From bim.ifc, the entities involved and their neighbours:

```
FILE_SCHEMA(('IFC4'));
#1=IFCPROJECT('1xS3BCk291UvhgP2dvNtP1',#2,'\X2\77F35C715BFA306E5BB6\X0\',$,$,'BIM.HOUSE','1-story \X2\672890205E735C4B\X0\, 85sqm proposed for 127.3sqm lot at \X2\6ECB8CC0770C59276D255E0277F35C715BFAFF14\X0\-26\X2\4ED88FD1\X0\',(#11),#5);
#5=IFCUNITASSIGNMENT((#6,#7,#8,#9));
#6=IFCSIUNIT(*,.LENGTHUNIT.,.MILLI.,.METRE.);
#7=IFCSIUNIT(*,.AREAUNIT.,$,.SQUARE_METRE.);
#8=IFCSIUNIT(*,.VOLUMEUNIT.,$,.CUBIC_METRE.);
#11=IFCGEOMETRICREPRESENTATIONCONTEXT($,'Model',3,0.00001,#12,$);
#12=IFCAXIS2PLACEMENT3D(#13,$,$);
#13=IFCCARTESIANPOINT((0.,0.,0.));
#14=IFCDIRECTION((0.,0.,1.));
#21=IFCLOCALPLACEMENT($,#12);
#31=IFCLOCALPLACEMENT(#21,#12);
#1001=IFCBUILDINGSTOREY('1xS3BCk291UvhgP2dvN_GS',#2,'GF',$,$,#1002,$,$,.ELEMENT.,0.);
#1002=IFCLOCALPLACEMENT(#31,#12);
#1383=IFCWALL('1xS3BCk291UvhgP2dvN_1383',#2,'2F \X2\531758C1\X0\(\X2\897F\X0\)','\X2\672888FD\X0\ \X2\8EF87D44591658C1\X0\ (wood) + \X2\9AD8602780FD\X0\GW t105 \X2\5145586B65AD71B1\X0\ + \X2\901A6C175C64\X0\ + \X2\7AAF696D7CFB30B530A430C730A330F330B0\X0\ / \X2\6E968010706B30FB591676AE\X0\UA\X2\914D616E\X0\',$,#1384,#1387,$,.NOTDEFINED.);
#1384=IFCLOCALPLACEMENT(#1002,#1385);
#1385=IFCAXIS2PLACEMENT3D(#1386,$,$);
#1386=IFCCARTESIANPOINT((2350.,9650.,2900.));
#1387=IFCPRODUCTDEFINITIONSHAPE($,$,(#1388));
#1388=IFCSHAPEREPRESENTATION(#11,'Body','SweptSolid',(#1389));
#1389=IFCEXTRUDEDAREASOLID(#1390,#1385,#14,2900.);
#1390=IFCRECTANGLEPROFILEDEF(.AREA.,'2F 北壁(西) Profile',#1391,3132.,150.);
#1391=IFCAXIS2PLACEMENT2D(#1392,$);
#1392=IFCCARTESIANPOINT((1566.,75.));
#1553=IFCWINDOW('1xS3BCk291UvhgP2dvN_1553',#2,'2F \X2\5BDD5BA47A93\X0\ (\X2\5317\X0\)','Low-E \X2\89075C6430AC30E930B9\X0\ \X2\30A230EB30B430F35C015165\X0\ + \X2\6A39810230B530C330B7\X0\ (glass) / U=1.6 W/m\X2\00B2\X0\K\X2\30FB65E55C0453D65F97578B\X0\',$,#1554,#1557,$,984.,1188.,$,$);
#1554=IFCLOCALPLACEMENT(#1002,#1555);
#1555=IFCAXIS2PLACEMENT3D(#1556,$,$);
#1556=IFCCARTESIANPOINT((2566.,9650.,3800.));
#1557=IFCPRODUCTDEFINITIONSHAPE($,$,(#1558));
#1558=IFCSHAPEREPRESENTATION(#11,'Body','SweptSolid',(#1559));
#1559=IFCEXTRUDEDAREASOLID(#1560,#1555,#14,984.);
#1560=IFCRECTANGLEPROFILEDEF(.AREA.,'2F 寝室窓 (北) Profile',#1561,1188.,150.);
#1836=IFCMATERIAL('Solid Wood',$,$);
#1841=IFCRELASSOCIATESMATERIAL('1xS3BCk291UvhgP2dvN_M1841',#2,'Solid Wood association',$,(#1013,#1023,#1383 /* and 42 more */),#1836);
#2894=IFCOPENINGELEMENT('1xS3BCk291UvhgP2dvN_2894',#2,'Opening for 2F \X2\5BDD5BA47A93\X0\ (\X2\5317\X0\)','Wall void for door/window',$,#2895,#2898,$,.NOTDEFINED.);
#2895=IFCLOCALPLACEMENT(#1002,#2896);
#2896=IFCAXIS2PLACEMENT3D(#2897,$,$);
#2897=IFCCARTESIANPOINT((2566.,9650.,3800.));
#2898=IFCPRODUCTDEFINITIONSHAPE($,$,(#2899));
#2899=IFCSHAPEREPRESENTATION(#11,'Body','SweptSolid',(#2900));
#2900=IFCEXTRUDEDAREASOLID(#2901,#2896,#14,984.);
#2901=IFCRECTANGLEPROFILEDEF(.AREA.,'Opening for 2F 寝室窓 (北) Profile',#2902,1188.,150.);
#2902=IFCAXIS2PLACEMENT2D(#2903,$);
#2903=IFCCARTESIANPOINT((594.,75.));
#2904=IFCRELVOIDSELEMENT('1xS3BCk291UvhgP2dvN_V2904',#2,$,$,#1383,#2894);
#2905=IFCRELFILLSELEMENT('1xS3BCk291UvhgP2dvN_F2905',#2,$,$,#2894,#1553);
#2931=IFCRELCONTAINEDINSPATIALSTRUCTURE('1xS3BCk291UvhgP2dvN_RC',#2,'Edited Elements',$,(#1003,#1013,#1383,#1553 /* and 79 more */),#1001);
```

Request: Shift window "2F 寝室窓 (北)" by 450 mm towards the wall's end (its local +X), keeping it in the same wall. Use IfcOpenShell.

```python
import ifcopenshell
import ifcopenshell.api.geometry
import ifcopenshell.util.placement
import ifcopenshell.util.unit

model = ifcopenshell.open("bim.ifc")
unit_scale = ifcopenshell.util.unit.calculate_unit_scale(model)

window = model.by_id(1553)
opening = window.FillsVoids[0].RelatingOpeningElement
wall = opening.VoidsElements[0].RelatingBuildingElement

wall_matrix = ifcopenshell.util.placement.get_local_placement(wall.ObjectPlacement)
shift = wall_matrix[:3, 0] * 0.45 / unit_scale
before = ifcopenshell.util.placement.get_local_placement(window.ObjectPlacement)[:3, 3].copy()

# The window is not placed relative to its opening, so move both.
for product in (opening, window):
    matrix = ifcopenshell.util.placement.get_local_placement(product.ObjectPlacement)
    matrix[:3, 3] += shift
    ifcopenshell.api.geometry.edit_object_placement(model, product=product, matrix=matrix, is_si=False)

after = ifcopenshell.util.placement.get_local_placement(window.ObjectPlacement)[:3, 3]
print("window moved by", (after - before).round(3) + 0.0)

model.write("bim_v2.ifc")
```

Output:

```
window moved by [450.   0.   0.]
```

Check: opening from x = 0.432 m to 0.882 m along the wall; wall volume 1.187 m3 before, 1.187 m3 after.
